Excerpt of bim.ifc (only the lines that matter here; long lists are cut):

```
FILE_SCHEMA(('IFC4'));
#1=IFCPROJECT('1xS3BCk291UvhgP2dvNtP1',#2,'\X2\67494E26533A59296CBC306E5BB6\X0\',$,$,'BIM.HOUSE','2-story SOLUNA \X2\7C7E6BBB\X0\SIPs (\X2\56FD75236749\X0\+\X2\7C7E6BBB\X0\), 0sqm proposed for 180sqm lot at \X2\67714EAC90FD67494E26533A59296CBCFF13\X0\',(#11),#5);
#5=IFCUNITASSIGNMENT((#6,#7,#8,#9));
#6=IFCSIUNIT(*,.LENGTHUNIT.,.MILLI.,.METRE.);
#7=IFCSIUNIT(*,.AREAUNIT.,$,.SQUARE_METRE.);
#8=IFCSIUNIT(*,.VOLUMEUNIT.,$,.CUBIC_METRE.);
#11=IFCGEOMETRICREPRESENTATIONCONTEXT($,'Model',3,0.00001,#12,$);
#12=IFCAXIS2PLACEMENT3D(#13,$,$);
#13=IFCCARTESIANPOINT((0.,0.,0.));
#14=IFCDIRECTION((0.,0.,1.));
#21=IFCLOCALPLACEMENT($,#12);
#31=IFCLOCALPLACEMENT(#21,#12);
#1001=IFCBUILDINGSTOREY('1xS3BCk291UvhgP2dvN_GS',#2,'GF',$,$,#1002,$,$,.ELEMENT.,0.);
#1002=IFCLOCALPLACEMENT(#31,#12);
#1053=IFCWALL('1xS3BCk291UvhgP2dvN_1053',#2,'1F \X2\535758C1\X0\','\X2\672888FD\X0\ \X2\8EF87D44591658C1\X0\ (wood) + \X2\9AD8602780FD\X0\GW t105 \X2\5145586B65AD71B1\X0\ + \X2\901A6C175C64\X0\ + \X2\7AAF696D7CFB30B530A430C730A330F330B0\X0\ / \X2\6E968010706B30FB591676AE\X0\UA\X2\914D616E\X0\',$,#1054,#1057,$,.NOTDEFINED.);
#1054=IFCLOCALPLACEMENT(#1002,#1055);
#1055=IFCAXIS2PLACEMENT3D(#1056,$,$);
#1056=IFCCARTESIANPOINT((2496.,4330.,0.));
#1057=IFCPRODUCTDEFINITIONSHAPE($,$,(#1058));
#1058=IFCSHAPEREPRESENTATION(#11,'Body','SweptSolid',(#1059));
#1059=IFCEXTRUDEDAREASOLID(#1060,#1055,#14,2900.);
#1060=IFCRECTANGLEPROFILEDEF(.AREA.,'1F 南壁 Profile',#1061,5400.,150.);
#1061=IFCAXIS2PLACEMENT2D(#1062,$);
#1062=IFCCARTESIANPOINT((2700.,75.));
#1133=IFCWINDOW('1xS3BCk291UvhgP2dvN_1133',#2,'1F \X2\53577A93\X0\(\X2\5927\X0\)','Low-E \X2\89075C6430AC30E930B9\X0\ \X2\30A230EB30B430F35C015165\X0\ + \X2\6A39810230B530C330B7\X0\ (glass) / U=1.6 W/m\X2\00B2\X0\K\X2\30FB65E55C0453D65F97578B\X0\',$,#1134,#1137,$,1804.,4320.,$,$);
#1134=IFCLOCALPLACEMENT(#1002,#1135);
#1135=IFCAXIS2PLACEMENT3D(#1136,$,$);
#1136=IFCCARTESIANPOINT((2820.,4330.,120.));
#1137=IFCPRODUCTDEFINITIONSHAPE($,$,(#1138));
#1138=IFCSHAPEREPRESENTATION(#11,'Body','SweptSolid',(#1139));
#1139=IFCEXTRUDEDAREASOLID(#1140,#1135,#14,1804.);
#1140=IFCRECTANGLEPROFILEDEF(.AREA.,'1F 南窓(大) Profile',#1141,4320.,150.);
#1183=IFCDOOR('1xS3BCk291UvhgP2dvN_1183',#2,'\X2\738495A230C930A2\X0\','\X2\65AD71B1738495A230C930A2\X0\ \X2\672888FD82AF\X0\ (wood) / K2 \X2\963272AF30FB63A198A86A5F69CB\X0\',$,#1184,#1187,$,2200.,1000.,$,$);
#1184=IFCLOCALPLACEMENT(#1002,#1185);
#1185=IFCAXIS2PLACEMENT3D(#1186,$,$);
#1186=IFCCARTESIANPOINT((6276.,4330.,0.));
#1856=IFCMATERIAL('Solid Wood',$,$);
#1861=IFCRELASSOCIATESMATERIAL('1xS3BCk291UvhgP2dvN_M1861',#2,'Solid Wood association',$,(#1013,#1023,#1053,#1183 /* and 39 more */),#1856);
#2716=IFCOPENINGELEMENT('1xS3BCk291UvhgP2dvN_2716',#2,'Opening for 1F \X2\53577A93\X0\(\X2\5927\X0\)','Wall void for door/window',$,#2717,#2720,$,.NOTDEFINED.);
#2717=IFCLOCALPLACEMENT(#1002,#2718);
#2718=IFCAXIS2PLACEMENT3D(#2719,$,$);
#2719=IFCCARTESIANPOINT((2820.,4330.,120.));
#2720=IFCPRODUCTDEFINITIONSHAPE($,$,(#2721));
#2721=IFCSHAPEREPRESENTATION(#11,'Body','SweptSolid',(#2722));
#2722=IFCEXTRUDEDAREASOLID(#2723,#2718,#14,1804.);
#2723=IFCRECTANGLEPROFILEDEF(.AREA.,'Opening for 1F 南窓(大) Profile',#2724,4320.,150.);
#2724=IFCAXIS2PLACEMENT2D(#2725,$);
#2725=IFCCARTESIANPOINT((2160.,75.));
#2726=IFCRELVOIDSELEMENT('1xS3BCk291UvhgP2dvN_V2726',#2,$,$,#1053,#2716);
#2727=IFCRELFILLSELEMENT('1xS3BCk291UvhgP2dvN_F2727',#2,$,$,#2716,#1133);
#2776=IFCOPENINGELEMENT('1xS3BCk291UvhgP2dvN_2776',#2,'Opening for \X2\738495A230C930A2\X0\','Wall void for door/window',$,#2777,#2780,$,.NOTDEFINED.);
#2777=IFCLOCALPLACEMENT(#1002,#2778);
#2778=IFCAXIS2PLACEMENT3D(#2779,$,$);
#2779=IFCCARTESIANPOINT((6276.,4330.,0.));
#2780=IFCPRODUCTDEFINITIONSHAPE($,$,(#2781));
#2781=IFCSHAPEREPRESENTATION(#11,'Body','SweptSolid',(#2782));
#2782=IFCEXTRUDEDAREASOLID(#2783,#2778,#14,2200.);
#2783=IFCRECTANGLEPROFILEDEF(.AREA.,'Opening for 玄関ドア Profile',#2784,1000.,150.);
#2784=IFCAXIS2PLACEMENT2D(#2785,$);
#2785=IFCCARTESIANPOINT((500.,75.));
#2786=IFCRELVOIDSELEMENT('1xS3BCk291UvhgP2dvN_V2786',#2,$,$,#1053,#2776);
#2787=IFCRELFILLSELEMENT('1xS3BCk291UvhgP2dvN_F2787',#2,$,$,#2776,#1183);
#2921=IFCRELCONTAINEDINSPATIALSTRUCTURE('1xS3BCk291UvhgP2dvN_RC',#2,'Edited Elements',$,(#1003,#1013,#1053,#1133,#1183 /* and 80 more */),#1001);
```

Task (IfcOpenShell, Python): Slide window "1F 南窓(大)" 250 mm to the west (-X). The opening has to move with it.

```python
import ifcopenshell
import ifcopenshell.api.geometry
import ifcopenshell.util.placement
import ifcopenshell.util.unit

model = ifcopenshell.open("bim.ifc")
unit_scale = ifcopenshell.util.unit.calculate_unit_scale(model)

window = model.by_id(1133)
opening = window.FillsVoids[0].RelatingOpeningElement
wall = opening.VoidsElements[0].RelatingBuildingElement

wall_matrix = ifcopenshell.util.placement.get_local_placement(wall.ObjectPlacement)
shift = wall_matrix[:3, 0] * -0.25 / unit_scale
before = ifcopenshell.util.placement.get_local_placement(window.ObjectPlacement)[:3, 3].copy()

# The window is not placed relative to its opening, so move both.
for product in (opening, window):
    matrix = ifcopenshell.util.placement.get_local_placement(product.ObjectPlacement)
    matrix[:3, 3] += shift
    ifcopenshell.api.geometry.edit_object_placement(model, product=product, matrix=matrix, is_si=False)

after = ifcopenshell.util.placement.get_local_placement(window.ObjectPlacement)[:3, 3]
print("window moved by", (after - before).round(3) + 0.0)

model.write("bim_v2.ifc")
```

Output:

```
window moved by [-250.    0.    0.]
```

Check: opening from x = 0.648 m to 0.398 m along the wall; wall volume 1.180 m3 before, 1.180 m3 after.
